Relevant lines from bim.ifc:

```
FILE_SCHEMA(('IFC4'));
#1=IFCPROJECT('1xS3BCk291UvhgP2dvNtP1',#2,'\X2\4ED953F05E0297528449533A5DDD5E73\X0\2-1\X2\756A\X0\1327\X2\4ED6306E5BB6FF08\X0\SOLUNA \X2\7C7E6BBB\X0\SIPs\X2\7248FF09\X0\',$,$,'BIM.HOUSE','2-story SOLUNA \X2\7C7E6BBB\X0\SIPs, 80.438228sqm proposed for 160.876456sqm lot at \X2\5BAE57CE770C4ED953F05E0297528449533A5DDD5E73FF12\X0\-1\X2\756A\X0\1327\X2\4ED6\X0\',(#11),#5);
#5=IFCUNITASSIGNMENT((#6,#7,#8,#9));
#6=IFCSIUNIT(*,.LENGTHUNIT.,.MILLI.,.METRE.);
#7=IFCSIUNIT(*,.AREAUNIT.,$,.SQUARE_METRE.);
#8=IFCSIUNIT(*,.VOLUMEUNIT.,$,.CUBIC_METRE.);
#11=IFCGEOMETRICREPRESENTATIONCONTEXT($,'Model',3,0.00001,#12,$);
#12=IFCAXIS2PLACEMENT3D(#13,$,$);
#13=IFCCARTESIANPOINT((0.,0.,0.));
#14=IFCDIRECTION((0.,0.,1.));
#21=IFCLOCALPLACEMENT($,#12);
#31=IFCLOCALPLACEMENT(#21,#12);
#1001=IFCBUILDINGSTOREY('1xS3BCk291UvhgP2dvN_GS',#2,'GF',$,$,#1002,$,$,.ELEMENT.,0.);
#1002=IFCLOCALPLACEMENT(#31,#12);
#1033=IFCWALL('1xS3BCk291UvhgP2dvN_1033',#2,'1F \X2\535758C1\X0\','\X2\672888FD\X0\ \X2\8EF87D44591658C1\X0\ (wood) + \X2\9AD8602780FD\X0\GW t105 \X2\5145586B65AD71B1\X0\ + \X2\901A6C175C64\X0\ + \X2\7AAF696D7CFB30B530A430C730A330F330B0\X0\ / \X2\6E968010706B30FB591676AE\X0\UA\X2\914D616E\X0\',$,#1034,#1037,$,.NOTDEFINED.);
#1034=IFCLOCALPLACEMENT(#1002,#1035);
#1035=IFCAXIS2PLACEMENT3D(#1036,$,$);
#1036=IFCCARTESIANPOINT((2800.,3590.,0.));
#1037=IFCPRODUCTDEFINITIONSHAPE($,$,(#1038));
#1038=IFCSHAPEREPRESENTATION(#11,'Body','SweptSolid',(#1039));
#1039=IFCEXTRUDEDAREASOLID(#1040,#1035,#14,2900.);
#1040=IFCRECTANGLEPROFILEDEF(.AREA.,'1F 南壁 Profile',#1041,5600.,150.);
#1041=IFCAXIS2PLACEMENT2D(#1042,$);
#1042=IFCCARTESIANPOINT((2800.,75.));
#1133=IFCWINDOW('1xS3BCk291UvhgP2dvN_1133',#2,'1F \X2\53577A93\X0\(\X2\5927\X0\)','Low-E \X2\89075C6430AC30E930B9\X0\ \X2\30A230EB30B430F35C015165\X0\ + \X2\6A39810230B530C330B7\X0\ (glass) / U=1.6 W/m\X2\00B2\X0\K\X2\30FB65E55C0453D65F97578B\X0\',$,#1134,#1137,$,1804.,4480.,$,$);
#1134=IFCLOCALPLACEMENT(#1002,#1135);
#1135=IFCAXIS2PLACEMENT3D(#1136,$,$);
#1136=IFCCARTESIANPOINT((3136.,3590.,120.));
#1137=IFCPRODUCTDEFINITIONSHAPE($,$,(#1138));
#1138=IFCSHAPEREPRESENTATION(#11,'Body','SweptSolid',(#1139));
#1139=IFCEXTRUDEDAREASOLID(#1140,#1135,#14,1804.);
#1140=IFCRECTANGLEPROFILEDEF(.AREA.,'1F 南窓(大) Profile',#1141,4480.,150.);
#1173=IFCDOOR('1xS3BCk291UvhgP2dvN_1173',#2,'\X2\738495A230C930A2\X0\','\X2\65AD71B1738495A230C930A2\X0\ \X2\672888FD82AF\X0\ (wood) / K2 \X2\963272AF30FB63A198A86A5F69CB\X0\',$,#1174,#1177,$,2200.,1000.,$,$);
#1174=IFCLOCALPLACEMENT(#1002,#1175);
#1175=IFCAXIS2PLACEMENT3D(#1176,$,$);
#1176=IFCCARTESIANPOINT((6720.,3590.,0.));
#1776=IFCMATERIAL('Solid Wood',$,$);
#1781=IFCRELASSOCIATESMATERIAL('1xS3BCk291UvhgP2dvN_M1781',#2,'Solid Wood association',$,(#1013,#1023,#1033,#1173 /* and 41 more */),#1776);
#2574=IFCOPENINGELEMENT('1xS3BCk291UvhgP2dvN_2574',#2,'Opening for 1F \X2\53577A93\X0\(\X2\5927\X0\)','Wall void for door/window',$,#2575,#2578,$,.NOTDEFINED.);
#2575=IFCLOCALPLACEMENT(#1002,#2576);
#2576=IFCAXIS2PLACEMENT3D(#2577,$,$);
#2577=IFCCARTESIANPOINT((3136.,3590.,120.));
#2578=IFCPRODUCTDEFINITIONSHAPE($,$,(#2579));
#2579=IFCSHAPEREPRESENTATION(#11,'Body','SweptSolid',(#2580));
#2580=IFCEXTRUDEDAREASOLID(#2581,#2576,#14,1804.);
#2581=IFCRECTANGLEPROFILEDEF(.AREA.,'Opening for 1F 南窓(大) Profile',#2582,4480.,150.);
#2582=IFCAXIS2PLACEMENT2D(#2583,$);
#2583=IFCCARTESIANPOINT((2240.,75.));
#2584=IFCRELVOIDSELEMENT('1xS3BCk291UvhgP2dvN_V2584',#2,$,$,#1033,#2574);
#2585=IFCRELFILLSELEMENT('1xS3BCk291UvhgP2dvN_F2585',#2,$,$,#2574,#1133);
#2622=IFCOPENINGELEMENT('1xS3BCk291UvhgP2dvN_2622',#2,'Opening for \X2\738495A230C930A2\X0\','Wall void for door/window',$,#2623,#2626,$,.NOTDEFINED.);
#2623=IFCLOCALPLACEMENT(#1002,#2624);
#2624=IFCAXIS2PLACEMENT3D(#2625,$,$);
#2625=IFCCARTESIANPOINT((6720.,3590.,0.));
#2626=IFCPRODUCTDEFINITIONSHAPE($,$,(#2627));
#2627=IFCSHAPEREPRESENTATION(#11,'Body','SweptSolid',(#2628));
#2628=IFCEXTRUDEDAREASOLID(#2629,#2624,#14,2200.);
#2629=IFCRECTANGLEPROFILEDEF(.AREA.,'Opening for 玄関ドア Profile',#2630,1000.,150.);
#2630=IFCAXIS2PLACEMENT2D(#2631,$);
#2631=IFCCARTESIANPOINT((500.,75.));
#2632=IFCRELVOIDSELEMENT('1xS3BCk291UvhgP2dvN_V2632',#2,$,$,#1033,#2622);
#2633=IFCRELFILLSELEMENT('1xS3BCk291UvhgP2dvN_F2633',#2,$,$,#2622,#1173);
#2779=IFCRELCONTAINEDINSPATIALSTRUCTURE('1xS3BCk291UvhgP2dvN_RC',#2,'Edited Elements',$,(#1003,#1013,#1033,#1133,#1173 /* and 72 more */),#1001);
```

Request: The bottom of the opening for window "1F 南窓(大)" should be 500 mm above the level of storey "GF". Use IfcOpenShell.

```python
import numpy as np
import ifcopenshell
import ifcopenshell.api.geometry
import ifcopenshell.geom
import ifcopenshell.util.element
import ifcopenshell.util.placement
import ifcopenshell.util.shape
import ifcopenshell.util.unit

model = ifcopenshell.open("bim.ifc")
unit_scale = ifcopenshell.util.unit.calculate_unit_scale(model)

window = model.by_guid("1xS3BCk291UvhgP2dvN_1133")
opening = window.FillsVoids[0].RelatingOpeningElement
storey = ifcopenshell.util.element.get_container(window, ifc_class="IfcBuildingStorey")
level = ifcopenshell.util.placement.get_local_placement(storey.ObjectPlacement)[2, 3]

# The opening's origin need not be at the sill, so measure its lowest point.
shape = ifcopenshell.geom.create_shape(ifcopenshell.geom.settings(), opening)
bottom = ifcopenshell.util.shape.get_shape_bottom_elevation(shape, shape.geometry) / unit_scale
dz = level + 0.5 / unit_scale - bottom

shift = np.array([0.0, 0.0, dz])
# The window is not placed relative to its opening, so move both.
for product in (opening, window):
    matrix = ifcopenshell.util.placement.get_local_placement(product.ObjectPlacement)
    matrix[:3, 3] += shift
    ifcopenshell.api.geometry.edit_object_placement(model, product=product, matrix=matrix, is_si=False)

print(f"moved by {dz * unit_scale:+.3f} m")

model.write("bim_v2.ifc")
```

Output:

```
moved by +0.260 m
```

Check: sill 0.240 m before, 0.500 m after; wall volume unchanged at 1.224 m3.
